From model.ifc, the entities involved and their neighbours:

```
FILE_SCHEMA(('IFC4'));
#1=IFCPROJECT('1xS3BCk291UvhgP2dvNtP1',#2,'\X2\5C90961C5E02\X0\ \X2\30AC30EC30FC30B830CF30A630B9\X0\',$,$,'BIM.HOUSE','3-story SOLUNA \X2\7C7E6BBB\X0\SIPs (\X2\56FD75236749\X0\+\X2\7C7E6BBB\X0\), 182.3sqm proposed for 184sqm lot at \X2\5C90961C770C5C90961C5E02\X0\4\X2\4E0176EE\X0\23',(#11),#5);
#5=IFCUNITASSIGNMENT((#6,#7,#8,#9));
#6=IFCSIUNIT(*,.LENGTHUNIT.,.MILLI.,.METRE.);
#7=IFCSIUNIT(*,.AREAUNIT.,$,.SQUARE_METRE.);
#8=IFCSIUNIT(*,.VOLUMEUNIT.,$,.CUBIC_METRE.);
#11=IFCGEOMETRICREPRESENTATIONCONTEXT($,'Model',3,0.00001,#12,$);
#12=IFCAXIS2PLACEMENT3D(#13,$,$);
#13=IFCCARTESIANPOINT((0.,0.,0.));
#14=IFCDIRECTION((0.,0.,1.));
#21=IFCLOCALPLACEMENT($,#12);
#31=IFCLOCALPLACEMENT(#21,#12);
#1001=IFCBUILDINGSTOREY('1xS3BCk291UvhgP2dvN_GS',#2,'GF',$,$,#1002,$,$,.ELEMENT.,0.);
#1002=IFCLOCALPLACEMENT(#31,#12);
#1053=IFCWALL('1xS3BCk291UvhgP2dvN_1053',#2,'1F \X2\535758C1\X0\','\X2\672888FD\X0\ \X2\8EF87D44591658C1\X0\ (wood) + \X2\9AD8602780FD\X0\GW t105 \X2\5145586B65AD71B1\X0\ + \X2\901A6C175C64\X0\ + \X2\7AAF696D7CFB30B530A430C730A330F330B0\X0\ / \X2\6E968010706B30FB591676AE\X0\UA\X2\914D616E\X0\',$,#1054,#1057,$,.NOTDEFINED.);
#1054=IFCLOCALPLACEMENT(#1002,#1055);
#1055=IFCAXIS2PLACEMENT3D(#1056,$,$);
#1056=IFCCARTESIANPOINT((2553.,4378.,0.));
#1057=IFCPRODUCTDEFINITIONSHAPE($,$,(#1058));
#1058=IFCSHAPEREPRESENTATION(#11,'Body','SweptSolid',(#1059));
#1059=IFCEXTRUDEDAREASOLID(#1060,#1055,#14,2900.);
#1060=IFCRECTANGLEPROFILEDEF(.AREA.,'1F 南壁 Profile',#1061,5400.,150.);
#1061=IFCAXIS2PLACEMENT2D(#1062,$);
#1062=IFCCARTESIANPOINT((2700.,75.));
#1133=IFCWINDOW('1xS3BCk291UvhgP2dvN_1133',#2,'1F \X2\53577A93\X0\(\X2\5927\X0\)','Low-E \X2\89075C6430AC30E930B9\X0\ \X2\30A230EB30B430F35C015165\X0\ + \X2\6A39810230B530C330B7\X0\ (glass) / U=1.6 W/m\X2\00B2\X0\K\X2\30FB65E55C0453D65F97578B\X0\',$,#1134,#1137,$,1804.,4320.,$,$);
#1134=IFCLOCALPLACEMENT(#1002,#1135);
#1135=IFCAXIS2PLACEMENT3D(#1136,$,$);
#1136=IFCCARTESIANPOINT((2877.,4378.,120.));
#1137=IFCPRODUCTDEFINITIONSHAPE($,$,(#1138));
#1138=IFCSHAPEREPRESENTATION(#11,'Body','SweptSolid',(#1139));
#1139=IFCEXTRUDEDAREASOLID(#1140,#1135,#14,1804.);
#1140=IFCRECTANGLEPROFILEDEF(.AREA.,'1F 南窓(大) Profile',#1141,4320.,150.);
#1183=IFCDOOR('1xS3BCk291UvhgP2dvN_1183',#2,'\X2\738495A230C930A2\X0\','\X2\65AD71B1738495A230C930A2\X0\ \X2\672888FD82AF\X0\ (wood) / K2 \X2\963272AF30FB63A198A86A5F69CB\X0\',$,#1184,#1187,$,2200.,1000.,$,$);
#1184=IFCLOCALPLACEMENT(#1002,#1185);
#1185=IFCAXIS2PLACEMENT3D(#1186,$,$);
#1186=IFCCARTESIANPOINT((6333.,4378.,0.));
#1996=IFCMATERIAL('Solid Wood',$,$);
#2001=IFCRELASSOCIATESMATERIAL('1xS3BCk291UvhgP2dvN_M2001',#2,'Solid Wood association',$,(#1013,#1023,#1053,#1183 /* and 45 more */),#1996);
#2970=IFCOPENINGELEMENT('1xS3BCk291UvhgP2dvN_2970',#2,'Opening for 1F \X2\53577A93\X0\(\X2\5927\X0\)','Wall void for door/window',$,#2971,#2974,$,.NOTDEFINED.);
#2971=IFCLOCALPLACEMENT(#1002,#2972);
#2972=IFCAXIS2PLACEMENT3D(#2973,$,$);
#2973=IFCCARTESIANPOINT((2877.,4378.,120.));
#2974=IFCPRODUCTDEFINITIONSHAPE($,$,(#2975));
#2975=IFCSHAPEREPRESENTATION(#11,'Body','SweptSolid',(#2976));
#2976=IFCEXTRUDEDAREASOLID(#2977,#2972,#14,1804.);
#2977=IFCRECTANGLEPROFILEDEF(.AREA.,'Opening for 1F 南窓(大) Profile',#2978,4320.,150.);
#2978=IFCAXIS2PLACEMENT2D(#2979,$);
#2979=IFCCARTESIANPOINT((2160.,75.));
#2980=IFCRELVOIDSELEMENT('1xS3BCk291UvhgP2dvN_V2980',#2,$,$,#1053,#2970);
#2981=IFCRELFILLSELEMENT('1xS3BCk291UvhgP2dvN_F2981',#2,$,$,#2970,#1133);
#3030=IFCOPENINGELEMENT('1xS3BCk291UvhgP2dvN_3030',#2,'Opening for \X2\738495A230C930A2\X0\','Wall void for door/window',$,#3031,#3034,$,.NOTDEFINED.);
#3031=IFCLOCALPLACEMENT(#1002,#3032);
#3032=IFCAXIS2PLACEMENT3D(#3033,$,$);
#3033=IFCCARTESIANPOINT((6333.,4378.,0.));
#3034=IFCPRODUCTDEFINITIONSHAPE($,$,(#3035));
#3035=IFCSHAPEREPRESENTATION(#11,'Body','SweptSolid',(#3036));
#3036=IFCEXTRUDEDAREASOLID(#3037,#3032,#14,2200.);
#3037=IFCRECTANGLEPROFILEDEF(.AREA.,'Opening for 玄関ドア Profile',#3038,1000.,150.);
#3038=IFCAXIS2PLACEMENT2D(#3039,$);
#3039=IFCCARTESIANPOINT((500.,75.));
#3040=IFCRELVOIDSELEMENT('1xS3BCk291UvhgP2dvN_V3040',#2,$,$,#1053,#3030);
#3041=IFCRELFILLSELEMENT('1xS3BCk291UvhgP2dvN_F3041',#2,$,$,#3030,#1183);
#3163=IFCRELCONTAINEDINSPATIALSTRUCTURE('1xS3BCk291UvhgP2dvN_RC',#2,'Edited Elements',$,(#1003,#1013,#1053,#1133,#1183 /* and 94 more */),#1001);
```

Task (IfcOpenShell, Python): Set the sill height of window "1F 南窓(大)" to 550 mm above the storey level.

```python
import numpy as np
import ifcopenshell
import ifcopenshell.api.geometry
import ifcopenshell.geom
import ifcopenshell.util.element
import ifcopenshell.util.placement
import ifcopenshell.util.shape
import ifcopenshell.util.unit

model = ifcopenshell.open("model.ifc")
unit_scale = ifcopenshell.util.unit.calculate_unit_scale(model)

window = model.by_guid("1xS3BCk291UvhgP2dvN_1133")
opening = window.FillsVoids[0].RelatingOpeningElement
storey = ifcopenshell.util.element.get_container(window, ifc_class="IfcBuildingStorey")
level = ifcopenshell.util.placement.get_local_placement(storey.ObjectPlacement)[2, 3]

# The opening's origin need not be at the sill, so measure its lowest point.
shape = ifcopenshell.geom.create_shape(ifcopenshell.geom.settings(), opening)
bottom = ifcopenshell.util.shape.get_shape_bottom_elevation(shape, shape.geometry) / unit_scale
dz = level + 550.0 - bottom

shift = np.array([0.0, 0.0, dz])
# The window is not placed relative to its opening, so move both.
for product in (opening, window):
    matrix = ifcopenshell.util.placement.get_local_placement(product.ObjectPlacement)
    matrix[:3, 3] += shift
    ifcopenshell.api.geometry.edit_object_placement(model, product=product, matrix=matrix, is_si=False)

print(f"moved by {dz * unit_scale:+.3f} m")

model.write("model_edited.ifc")
```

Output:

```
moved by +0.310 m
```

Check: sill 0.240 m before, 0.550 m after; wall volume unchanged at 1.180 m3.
